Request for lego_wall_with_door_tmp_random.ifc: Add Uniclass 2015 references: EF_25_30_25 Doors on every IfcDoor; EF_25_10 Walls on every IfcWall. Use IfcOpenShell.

First a look at what the model holds.

```python
import ifcopenshell

model = ifcopenshell.open("lego_wall_with_door_tmp_random.ifc")
print(model.schema)
print("classifications:", [c.Name for c in model.by_type("IfcClassification")])
for ifc_class in ("IfcDoor", "IfcRoof", "IfcStair", "IfcWall", "IfcWindow"):
    print(ifc_class, len(model.by_type(ifc_class)))
```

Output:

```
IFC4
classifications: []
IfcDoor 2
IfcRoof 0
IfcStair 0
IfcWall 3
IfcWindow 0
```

```python
import ifcopenshell
import ifcopenshell.api.classification

model = ifcopenshell.open("lego_wall_with_door_tmp_random.ifc")

system = ifcopenshell.api.classification.add_classification(model, classification="Uniclass 2015")

codes = {
    "IfcDoor": ("EF_25_30_25", "Doors"),
    "IfcWall": ("EF_25_10", "Walls"),
}
for ifc_class, (code, name) in codes.items():
    products = model.by_type(ifc_class)
    ifcopenshell.api.classification.add_reference(
        model, products=products, classification=system, identification=code, name=name
    )
    print(code, len(products))

model.write("lego_wall_with_door_tmp_random-out.ifc")
```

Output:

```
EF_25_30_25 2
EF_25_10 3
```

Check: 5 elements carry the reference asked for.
